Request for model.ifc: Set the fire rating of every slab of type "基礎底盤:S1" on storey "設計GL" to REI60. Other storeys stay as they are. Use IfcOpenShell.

First a look at what the model holds.

```python
import ifcopenshell
import ifcopenshell.util.element

model = ifcopenshell.open("model.ifc")
print(model.schema)
storey = next(s for s in model.by_type("IfcBuildingStorey") if s.Name == "設計GL")
slabs = [e for e in ifcopenshell.util.element.get_decomposition(storey) if e.is_a("IfcSlab")]
seen = {}
for e in slabs:
    element_type = ifcopenshell.util.element.get_type(e)
    key = (element_type.Name if element_type != e and element_type else None, ifcopenshell.util.element.get_pset(e, "Pset_SlabCommon", "FireRating"))
    seen[key] = seen.get(key, 0) + 1
for (name, value), count in sorted(seen.items(), key=str):
    print(count, "x", name, "|", value)
```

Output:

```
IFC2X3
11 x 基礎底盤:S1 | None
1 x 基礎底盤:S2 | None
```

```python
import ifcopenshell
import ifcopenshell.api.pset
import ifcopenshell.util.element

model = ifcopenshell.open("model.ifc")

storey = next(s for s in model.by_type("IfcBuildingStorey") if s.Name == "設計GL")
slabs = [e for e in ifcopenshell.util.element.get_decomposition(storey) if e.is_a("IfcSlab")]

count = 0
for e in slabs:
    element_type = ifcopenshell.util.element.get_type(e)
    if element_type in (None, e) or element_type.Name != "基礎底盤:S1":
        continue
    # add_pset returns the element's existing set when there is one.
    pset = ifcopenshell.api.pset.add_pset(model, product=e, name="Pset_SlabCommon")
    ifcopenshell.api.pset.edit_pset(model, pset=pset, properties={"FireRating": "REI60"})
    count += 1

print(count, "slabs updated")

model.write("model_updated.ifc")
```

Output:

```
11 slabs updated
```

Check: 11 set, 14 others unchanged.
